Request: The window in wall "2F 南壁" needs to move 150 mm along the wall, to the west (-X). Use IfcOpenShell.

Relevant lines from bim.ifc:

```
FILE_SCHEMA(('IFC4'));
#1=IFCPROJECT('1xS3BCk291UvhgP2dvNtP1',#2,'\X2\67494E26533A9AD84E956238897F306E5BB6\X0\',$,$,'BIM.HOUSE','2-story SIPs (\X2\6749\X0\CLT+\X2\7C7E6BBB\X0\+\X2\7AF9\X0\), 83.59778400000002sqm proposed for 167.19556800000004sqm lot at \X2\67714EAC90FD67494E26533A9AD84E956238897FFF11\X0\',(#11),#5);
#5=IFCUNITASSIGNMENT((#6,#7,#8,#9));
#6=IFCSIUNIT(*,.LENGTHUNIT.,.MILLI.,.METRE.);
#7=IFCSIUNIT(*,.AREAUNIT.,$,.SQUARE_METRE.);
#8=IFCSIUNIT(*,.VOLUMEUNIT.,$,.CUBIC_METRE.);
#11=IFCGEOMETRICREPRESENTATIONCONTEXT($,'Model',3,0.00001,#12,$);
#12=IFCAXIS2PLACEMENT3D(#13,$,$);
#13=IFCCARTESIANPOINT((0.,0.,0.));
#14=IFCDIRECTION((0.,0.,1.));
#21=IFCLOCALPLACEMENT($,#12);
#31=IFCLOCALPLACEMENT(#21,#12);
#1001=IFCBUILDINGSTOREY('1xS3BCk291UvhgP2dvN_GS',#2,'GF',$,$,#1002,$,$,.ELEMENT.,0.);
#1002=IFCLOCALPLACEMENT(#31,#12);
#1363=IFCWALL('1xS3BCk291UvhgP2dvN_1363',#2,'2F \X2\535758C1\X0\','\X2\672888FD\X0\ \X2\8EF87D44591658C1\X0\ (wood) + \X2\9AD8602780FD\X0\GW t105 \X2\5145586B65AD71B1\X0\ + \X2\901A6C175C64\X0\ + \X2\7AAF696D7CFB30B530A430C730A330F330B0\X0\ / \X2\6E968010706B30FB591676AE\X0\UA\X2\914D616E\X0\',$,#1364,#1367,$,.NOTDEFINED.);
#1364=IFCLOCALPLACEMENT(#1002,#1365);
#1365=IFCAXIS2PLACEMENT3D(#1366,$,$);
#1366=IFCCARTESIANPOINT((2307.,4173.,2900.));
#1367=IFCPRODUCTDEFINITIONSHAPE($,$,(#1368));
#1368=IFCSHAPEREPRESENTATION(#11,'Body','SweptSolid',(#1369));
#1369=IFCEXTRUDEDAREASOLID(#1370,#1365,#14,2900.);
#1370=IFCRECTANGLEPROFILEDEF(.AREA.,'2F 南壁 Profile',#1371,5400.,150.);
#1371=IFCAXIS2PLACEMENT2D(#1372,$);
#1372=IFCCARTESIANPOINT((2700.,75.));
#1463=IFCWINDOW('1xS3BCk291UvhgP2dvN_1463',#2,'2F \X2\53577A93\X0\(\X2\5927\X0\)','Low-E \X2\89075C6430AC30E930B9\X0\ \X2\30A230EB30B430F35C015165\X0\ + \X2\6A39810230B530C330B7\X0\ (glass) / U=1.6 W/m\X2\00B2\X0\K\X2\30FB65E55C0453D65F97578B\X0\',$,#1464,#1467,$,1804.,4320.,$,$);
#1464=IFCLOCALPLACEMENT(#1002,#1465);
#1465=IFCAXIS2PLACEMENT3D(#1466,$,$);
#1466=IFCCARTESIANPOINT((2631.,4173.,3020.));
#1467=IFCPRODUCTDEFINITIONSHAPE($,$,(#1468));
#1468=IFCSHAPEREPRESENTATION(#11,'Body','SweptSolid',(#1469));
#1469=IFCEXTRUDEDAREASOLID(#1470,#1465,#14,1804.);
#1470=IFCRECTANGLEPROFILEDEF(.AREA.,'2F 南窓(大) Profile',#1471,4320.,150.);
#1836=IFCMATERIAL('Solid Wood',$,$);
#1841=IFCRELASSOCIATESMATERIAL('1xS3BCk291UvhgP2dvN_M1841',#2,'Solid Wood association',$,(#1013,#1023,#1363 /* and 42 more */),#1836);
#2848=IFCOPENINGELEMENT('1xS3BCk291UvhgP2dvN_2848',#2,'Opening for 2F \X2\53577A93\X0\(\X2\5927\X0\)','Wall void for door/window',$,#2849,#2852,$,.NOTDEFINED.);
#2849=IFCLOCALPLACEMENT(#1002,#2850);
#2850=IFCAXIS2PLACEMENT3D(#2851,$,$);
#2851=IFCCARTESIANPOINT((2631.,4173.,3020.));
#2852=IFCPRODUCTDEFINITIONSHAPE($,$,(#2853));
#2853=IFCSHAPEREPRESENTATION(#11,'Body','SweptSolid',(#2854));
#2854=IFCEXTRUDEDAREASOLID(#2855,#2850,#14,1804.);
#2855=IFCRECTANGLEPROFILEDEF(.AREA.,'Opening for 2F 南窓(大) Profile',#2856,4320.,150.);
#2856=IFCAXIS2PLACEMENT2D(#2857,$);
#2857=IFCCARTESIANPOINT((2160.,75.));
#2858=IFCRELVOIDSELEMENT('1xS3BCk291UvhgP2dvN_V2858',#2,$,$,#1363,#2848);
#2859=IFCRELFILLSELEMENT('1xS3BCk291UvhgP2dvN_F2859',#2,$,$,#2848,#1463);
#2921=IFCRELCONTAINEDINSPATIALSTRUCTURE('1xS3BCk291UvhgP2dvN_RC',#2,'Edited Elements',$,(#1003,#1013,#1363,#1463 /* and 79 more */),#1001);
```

```python
import ifcopenshell
import ifcopenshell.api.geometry
import ifcopenshell.util.placement
import ifcopenshell.util.unit

model = ifcopenshell.open("bim.ifc")
unit_scale = ifcopenshell.util.unit.calculate_unit_scale(model)

window = model.by_id(1463)
opening = window.FillsVoids[0].RelatingOpeningElement
wall = opening.VoidsElements[0].RelatingBuildingElement

wall_matrix = ifcopenshell.util.placement.get_local_placement(wall.ObjectPlacement)
shift = wall_matrix[:3, 0] * -0.15 / unit_scale
before = ifcopenshell.util.placement.get_local_placement(window.ObjectPlacement)[:3, 3].copy()

# The window is not placed relative to its opening, so move both.
for product in (opening, window):
    matrix = ifcopenshell.util.placement.get_local_placement(product.ObjectPlacement)
    matrix[:3, 3] += shift
    ifcopenshell.api.geometry.edit_object_placement(model, product=product, matrix=matrix, is_si=False)

after = ifcopenshell.util.placement.get_local_placement(window.ObjectPlacement)[:3, 3]
print("window moved by", (after - before).round(3) + 0.0)

model.write("bim_edited.ifc")
```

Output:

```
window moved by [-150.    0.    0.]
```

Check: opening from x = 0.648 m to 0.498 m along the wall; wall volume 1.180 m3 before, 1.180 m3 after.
